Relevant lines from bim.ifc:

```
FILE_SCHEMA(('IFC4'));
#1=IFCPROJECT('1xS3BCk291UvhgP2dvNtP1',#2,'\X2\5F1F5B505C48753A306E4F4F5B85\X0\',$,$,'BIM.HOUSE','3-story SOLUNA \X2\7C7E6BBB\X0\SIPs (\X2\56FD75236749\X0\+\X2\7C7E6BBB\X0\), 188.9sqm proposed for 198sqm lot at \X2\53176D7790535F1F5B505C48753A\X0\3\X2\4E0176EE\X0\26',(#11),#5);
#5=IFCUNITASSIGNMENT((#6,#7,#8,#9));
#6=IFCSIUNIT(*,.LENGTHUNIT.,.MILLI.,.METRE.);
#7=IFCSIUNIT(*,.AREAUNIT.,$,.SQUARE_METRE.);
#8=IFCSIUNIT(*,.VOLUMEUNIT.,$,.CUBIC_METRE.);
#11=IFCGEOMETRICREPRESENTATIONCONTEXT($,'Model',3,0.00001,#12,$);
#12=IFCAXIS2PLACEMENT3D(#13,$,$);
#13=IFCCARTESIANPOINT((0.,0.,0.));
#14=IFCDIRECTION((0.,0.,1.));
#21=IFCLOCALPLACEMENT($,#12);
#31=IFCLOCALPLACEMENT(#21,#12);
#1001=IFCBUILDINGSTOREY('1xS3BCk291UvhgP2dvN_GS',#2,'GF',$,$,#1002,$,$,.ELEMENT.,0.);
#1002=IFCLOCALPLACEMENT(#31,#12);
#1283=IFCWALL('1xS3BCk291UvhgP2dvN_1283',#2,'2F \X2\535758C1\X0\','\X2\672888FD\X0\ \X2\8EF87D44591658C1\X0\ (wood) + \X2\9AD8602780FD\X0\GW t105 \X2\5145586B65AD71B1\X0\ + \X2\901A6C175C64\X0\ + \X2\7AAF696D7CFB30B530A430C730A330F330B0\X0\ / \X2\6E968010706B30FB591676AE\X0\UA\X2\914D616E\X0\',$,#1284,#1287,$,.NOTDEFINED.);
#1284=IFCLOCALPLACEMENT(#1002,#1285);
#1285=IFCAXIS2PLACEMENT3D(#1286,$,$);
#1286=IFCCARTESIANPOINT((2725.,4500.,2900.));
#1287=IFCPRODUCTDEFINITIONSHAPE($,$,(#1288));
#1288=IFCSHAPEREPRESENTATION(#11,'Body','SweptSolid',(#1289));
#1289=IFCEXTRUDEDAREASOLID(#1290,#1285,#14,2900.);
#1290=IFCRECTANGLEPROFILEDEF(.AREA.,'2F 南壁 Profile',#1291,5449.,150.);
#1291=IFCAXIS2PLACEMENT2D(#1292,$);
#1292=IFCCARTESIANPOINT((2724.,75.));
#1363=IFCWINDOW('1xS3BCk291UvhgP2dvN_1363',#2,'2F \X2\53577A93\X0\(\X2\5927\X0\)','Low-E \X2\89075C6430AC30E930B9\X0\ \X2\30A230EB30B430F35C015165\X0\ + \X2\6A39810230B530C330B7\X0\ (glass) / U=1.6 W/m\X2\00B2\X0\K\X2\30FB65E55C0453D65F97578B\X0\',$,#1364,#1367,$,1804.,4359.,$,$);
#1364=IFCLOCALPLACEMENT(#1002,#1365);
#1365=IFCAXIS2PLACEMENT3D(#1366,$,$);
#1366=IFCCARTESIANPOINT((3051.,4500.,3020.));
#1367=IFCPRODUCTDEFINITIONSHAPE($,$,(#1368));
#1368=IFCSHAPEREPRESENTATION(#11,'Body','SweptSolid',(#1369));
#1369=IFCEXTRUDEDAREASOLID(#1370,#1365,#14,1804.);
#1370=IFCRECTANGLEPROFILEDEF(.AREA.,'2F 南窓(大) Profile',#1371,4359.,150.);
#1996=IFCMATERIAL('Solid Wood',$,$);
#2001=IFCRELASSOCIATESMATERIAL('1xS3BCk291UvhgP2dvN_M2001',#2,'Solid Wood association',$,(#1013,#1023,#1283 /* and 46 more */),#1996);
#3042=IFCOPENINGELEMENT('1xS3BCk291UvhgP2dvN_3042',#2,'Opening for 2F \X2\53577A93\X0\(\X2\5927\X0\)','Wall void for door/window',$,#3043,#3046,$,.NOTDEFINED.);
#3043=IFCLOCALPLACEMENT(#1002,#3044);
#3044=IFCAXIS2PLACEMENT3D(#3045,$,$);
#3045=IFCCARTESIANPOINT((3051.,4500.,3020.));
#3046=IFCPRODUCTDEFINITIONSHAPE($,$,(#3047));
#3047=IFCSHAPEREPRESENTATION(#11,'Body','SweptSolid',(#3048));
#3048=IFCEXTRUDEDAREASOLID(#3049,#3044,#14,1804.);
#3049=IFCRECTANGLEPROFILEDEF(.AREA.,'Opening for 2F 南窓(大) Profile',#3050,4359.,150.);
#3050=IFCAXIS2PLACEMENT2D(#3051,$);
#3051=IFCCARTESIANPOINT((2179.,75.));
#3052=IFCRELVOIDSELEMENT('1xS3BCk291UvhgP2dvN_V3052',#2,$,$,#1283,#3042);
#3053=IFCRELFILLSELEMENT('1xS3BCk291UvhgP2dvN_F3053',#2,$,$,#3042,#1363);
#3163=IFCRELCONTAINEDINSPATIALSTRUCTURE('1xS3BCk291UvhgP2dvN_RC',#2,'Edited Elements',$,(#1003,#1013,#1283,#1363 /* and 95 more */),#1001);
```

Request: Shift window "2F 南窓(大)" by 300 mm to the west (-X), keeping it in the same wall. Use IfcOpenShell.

```python
import ifcopenshell
import ifcopenshell.api.geometry
import ifcopenshell.util.placement
import ifcopenshell.util.unit

model = ifcopenshell.open("bim.ifc")
unit_scale = ifcopenshell.util.unit.calculate_unit_scale(model)

window = model.by_id(1363)
opening = window.FillsVoids[0].RelatingOpeningElement
wall = opening.VoidsElements[0].RelatingBuildingElement

wall_matrix = ifcopenshell.util.placement.get_local_placement(wall.ObjectPlacement)
shift = wall_matrix[:3, 0] * -0.3 / unit_scale
before = ifcopenshell.util.placement.get_local_placement(window.ObjectPlacement)[:3, 3].copy()

# The window is not placed relative to its opening, so move both.
for product in (opening, window):
    matrix = ifcopenshell.util.placement.get_local_placement(product.ObjectPlacement)
    matrix[:3, 3] += shift
    ifcopenshell.api.geometry.edit_object_placement(model, product=product, matrix=matrix, is_si=False)

after = ifcopenshell.util.placement.get_local_placement(window.ObjectPlacement)[:3, 3]
print("window moved by", (after - before).round(3) + 0.0)

model.write("bim_v2.ifc")
```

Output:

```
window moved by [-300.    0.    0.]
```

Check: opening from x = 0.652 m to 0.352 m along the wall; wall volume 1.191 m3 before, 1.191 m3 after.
